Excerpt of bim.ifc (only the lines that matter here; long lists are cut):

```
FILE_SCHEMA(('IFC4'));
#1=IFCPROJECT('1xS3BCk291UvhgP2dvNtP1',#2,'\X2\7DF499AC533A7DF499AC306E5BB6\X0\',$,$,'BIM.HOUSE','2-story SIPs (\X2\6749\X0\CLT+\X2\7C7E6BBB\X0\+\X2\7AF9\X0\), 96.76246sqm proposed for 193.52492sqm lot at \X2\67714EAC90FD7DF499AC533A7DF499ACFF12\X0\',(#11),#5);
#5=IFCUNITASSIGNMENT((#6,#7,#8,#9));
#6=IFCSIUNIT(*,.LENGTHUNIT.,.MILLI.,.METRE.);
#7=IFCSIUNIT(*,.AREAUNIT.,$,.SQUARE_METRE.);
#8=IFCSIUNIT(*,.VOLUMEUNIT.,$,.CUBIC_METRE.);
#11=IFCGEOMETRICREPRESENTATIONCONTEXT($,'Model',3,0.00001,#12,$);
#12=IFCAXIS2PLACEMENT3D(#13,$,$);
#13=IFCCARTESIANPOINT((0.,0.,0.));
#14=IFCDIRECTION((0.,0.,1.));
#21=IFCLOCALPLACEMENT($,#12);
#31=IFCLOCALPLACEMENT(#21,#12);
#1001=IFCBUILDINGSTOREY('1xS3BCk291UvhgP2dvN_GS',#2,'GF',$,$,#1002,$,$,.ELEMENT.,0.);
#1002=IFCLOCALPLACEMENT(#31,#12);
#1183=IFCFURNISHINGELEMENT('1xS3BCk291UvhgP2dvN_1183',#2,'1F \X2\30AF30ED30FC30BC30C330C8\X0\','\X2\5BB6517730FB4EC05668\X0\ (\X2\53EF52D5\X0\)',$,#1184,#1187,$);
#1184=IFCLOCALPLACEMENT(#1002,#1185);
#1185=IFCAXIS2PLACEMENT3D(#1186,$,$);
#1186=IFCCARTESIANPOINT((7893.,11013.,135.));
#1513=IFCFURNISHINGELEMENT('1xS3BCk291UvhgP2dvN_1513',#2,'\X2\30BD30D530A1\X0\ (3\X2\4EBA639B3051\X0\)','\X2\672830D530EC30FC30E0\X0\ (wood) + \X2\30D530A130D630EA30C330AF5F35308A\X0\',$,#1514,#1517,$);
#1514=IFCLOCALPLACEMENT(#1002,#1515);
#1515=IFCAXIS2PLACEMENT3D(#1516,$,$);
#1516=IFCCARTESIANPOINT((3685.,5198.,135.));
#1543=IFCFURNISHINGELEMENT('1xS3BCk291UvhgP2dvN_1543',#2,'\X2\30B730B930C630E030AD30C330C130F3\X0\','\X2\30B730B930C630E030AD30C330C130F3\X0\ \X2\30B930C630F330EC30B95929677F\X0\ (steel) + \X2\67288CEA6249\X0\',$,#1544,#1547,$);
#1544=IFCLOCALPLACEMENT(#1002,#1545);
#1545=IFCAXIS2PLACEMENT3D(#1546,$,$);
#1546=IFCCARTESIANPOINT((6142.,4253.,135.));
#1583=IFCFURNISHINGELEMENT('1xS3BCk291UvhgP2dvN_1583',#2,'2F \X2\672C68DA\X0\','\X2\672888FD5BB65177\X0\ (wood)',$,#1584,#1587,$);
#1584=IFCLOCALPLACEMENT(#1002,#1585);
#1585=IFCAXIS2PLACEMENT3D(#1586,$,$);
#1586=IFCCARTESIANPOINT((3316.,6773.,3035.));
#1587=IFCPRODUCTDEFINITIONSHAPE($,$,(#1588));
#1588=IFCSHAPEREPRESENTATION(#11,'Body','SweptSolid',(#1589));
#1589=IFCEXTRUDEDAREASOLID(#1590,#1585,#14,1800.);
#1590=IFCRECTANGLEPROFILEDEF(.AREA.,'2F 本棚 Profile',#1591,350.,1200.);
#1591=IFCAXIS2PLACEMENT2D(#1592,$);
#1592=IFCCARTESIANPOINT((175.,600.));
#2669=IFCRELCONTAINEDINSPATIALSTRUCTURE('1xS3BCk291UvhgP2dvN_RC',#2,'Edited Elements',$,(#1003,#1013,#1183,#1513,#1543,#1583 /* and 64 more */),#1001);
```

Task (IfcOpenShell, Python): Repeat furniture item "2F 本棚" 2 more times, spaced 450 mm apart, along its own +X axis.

```python
import ifcopenshell
import ifcopenshell.api.geometry
import ifcopenshell.api.root
import ifcopenshell.util.element
import ifcopenshell.util.placement

model = ifcopenshell.open("bim.ifc")


def reuse_history(source, copy):
    """copy_class also copies each property set's owner history, people and application; keep the originals."""
    for rel in copy.IsDefinedBy:
        if rel.is_a("IfcRelDefinesByProperties") and (history := rel.RelatingPropertyDefinition.OwnerHistory):
            rel.RelatingPropertyDefinition.OwnerHistory = source.OwnerHistory
            ifcopenshell.util.element.remove_deep2(model, history)


source = model.by_guid("1xS3BCk291UvhgP2dvN_1583")
base = ifcopenshell.util.placement.get_local_placement(source.ObjectPlacement)
step = base[:3, 0] * 450.0

for i in range(1, 3):
    copy = ifcopenshell.api.root.copy_class(model, product=source)
    copy.Representation = ifcopenshell.util.element.copy_deep(
        model, source.Representation, exclude=["IfcGeometricRepresentationContext", "IfcRepresentationMap"]
    )
    reuse_history(source, copy)
    matrix = base.copy()
    matrix[:3, 3] += i * step
    print("added at", matrix[:3, 3].round(3) + 0.0)
    ifcopenshell.api.geometry.edit_object_placement(model, product=copy, matrix=matrix, is_si=False)

model.write("bim_edited.ifc")
```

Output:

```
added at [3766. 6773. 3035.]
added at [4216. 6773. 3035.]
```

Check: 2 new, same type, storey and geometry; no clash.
